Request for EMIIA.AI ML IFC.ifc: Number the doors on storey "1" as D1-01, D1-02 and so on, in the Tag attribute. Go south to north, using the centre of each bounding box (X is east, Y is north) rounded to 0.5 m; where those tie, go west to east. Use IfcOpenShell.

First a look at what the model holds.

```python
import ifcopenshell
import ifcopenshell.util.element
import ifcopenshell.util.placement

model = ifcopenshell.open("EMIIA.AI ML IFC.ifc")
print(model.schema)
storey = next(s for s in model.by_type("IfcBuildingStorey") if s.Name == "1")
doors = [e for e in ifcopenshell.util.element.get_decomposition(storey) if e.is_a("IfcDoor")]
for e in sorted(doors, key=lambda e: e.id()):
    origin = ifcopenshell.util.placement.get_local_placement(e.ObjectPlacement)[:3, 3]
    print(e.id(), e.Tag, e.Name, origin.round(2) + 0.0, sep=" | ")
```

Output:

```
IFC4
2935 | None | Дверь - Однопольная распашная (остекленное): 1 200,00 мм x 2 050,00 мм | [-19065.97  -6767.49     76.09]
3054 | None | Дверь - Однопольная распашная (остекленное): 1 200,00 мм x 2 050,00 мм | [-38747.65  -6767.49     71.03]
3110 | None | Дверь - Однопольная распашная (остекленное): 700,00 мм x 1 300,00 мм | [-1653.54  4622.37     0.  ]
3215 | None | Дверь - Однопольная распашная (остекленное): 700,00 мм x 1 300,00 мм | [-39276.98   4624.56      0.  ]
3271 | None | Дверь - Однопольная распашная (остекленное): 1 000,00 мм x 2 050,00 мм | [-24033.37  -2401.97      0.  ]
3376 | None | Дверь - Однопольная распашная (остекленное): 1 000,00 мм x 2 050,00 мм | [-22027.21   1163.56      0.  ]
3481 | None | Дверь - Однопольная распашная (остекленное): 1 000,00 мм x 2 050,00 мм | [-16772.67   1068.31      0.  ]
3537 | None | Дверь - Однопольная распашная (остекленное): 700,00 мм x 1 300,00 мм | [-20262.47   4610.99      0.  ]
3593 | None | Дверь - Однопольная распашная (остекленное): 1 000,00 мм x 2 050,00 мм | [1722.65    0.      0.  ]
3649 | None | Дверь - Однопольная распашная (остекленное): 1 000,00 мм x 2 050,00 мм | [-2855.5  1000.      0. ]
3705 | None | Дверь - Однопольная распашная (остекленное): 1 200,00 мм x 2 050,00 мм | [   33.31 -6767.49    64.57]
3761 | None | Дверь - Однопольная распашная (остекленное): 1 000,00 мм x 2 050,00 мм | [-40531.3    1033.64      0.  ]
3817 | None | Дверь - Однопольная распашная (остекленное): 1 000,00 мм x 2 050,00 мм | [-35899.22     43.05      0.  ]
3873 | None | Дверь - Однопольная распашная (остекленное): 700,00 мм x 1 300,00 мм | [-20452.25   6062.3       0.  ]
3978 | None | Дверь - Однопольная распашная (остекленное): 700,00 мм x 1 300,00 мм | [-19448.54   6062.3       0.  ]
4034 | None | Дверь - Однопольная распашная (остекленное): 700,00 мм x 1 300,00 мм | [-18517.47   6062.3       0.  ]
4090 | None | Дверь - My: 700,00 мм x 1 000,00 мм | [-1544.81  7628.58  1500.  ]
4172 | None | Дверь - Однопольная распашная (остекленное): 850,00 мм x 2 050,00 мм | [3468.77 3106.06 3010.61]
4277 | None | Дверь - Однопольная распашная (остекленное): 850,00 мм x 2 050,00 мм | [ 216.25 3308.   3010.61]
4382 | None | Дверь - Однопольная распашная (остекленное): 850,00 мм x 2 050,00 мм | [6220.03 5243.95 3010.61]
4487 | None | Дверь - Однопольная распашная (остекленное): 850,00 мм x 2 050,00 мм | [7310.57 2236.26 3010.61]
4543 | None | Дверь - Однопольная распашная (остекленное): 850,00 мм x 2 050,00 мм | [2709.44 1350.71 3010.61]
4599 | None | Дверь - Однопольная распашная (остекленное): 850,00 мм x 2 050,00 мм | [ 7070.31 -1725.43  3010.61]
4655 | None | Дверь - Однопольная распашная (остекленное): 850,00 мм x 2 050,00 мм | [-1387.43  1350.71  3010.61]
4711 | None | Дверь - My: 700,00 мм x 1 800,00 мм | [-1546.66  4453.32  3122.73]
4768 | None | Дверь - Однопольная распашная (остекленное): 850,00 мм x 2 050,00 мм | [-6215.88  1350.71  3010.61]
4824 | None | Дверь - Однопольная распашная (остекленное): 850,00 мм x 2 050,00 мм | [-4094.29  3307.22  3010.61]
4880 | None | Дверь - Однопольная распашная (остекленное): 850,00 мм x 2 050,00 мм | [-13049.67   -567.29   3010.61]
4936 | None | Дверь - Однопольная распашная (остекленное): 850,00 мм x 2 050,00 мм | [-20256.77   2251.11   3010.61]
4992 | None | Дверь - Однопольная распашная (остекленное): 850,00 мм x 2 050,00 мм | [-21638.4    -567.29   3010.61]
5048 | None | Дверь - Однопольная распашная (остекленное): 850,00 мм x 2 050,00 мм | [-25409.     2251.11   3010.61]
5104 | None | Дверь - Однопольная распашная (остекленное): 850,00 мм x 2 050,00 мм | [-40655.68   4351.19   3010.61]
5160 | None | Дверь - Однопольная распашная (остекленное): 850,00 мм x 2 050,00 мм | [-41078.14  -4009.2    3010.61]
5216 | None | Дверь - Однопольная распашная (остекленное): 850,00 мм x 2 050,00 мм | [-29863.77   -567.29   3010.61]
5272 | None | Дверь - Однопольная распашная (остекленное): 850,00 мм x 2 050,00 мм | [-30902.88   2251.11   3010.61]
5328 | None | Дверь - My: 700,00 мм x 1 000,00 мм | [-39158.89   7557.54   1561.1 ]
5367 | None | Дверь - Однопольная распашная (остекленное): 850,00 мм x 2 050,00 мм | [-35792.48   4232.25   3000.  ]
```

```python
import ifcopenshell
import ifcopenshell.geom
import ifcopenshell.util.element
import ifcopenshell.util.shape

model = ifcopenshell.open("EMIIA.AI ML IFC.ifc")
settings = ifcopenshell.geom.settings()
settings.set("use-world-coords", True)


def centre(element):
    shape = ifcopenshell.geom.create_shape(settings, element)
    return ifcopenshell.util.shape.get_bbox_centroid(shape.geometry)


storey = next(s for s in model.by_type("IfcBuildingStorey") if s.Name == "1")
doors = [e for e in ifcopenshell.util.element.get_decomposition(storey) if e.is_a("IfcDoor")]

# Insertion points can sit at a corner or the storey origin, so sort by the geometry (in metres).
centres = {e: centre(e) for e in doors}
doors.sort(key=lambda e: (round(centres[e][1] / 0.5), centres[e][0]))

for i, e in enumerate(doors, start=1):
    number = f"D1-{i:02d}"
    e.Tag = number
    print(e.id(), number)

model.write("EMIIA.AI ML IFC_v2.ifc")
```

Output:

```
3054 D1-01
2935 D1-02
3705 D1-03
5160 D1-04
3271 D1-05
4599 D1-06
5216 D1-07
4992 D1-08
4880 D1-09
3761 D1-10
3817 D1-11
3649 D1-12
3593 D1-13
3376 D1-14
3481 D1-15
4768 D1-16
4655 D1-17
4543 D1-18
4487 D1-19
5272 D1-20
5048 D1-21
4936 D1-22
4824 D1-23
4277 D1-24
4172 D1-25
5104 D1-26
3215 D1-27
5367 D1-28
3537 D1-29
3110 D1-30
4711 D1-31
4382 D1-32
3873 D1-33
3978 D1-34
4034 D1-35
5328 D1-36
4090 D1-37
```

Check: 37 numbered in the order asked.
